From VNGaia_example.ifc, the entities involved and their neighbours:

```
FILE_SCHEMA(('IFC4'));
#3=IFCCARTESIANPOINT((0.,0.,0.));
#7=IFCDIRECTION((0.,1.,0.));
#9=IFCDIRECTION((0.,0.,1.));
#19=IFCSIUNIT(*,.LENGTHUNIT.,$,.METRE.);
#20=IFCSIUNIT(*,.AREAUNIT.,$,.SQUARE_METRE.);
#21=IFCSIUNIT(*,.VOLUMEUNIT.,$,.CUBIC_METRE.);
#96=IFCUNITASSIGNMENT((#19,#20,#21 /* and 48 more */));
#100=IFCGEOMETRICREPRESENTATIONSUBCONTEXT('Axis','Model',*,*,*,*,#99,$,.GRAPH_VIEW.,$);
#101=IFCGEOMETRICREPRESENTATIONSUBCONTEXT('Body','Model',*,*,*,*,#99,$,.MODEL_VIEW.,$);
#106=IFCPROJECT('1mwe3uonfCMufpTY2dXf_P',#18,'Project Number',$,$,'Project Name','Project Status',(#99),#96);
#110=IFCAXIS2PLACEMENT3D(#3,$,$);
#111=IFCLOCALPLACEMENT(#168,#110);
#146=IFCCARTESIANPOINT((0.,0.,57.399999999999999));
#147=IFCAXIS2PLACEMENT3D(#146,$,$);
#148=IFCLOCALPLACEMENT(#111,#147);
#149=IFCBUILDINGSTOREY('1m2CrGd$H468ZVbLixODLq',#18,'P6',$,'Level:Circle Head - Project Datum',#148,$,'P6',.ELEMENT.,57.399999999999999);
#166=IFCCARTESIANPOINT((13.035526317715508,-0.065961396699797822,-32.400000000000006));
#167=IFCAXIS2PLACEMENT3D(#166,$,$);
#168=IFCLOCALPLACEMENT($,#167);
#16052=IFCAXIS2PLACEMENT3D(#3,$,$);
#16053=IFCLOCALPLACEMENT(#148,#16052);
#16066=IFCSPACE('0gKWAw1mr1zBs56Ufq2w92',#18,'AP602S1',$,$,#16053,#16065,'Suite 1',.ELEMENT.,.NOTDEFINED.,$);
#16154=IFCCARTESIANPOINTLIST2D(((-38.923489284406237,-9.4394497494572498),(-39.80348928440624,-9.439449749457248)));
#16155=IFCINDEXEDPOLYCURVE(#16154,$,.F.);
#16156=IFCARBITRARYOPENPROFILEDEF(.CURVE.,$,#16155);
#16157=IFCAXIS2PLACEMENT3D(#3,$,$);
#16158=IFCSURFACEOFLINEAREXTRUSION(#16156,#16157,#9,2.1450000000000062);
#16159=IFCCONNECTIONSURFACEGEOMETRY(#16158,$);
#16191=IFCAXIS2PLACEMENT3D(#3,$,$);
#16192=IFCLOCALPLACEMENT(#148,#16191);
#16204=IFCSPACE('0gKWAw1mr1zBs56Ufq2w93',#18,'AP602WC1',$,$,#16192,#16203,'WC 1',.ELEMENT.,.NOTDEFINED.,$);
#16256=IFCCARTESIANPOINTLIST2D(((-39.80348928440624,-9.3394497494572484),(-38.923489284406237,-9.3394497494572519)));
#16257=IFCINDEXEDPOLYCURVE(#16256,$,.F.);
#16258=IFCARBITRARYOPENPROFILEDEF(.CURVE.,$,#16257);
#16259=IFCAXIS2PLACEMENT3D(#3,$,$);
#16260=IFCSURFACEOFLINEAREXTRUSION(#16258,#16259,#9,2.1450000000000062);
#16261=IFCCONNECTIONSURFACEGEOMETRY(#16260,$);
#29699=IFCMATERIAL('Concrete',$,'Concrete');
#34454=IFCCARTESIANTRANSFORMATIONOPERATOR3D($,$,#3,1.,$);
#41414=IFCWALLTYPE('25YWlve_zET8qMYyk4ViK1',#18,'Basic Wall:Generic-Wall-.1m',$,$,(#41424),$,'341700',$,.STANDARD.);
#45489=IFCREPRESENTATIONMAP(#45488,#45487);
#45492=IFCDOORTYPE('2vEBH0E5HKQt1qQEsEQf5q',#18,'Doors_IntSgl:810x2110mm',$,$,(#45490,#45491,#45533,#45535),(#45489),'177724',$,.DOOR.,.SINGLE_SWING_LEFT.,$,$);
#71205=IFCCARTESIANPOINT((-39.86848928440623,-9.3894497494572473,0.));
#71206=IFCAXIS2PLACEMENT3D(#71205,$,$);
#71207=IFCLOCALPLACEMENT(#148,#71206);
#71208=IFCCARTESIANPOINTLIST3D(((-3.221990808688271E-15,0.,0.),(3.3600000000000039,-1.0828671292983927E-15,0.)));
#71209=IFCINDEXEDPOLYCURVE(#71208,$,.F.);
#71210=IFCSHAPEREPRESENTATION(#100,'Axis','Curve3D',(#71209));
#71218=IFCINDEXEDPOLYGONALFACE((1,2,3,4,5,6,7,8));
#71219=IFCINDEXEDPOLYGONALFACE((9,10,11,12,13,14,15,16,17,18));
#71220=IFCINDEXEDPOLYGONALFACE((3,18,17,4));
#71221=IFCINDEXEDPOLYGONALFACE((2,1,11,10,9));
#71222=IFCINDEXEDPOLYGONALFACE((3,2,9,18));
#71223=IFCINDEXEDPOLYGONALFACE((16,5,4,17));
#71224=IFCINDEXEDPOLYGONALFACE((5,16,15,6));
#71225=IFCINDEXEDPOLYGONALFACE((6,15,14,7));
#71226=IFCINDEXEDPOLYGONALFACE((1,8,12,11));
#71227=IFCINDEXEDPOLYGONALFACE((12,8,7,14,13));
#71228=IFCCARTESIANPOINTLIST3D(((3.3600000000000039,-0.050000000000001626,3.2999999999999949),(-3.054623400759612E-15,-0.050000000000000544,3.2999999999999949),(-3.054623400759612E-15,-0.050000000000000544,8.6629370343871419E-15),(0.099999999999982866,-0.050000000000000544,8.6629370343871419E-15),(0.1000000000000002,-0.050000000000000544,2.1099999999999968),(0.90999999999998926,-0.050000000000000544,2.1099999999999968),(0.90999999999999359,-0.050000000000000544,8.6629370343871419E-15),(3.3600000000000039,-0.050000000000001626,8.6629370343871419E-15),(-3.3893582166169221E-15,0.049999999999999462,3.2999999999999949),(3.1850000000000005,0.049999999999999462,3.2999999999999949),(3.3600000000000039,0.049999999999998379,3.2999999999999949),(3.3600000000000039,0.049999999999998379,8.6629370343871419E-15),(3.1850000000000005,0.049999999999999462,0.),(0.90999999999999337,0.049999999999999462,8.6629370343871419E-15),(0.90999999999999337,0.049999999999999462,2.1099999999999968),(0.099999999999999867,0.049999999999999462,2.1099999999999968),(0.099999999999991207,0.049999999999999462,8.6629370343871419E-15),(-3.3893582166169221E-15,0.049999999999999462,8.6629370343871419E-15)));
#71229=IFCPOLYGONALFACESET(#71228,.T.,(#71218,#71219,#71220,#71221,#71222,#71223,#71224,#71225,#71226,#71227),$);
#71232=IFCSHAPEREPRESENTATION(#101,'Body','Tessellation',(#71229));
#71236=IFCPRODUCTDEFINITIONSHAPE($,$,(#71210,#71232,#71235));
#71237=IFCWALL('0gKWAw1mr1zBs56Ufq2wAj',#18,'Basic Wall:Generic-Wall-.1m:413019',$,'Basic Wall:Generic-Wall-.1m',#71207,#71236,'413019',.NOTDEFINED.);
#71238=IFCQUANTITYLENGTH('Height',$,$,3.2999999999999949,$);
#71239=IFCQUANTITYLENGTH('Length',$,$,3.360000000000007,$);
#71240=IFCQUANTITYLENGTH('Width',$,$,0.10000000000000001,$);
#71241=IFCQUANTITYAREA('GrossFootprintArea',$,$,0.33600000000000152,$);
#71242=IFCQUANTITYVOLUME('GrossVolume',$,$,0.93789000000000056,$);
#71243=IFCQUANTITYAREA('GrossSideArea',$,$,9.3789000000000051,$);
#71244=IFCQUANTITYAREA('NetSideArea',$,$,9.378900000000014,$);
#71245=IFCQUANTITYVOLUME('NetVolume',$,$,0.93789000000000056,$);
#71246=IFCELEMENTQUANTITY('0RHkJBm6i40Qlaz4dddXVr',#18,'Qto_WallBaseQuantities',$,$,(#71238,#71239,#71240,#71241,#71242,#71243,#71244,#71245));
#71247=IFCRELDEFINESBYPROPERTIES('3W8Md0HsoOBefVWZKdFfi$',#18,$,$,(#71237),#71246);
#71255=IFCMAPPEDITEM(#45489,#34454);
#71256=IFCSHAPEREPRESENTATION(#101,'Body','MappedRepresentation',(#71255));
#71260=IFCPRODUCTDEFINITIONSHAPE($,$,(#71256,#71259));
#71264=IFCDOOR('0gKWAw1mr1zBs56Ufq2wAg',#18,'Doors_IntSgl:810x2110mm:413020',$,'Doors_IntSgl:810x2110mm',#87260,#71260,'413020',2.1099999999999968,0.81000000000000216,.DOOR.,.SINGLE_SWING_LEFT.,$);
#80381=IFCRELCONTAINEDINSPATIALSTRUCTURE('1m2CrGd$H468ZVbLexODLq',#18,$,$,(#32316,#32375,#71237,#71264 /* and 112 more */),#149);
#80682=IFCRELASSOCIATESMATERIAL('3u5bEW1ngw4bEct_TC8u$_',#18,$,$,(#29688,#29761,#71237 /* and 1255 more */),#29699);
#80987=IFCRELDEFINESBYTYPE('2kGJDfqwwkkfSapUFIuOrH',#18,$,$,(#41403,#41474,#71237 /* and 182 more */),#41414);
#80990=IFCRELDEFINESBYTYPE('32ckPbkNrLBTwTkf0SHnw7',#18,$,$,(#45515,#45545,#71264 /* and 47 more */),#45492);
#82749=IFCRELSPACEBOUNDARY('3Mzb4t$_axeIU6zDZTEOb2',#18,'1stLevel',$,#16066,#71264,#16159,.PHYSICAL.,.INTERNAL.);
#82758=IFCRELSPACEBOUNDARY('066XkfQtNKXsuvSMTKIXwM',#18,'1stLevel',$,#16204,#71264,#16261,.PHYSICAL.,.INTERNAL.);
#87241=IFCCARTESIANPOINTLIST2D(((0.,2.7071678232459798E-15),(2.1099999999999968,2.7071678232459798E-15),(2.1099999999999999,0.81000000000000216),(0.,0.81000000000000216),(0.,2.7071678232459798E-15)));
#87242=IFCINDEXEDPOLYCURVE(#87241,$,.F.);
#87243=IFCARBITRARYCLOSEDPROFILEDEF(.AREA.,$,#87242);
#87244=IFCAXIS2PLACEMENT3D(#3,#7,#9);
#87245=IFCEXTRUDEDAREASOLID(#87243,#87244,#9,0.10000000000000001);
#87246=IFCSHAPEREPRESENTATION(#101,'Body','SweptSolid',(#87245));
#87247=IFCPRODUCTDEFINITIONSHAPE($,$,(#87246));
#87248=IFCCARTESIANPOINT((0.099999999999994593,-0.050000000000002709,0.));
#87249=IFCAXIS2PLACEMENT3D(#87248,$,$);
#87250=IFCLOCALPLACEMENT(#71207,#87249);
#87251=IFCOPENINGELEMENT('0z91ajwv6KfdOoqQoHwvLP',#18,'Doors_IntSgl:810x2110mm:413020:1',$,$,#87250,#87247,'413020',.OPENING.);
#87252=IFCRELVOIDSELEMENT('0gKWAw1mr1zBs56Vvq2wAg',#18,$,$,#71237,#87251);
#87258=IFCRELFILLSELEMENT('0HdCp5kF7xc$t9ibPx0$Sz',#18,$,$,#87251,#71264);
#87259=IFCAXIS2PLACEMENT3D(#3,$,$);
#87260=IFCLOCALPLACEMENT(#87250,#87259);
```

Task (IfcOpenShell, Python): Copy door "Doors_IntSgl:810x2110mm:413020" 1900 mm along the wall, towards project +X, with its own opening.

```python
import numpy as np
import ifcopenshell
import ifcopenshell.api.feature
import ifcopenshell.api.geometry
import ifcopenshell.api.pset
import ifcopenshell.api.root
import ifcopenshell.geom
import ifcopenshell.util.element
import ifcopenshell.util.placement
import ifcopenshell.util.shape
import ifcopenshell.util.unit

model = ifcopenshell.open("VNGaia_example.ifc")
area_scale = ifcopenshell.util.unit.calculate_unit_scale(model, "AREAUNIT")
volume_scale = ifcopenshell.util.unit.calculate_unit_scale(model, "VOLUMEUNIT")
settings = ifcopenshell.geom.settings()


def volume(element):
    """Net volume in cubic metres, openings subtracted."""
    shape = ifcopenshell.geom.create_shape(settings, element)
    return ifcopenshell.util.shape.get_volume(shape.geometry)


def reuse_history(source, copy):
    """copy_class also copies each property set's owner history, people and application; keep the originals."""
    for rel in copy.IsDefinedBy:
        if rel.is_a("IfcRelDefinesByProperties") and (history := rel.RelatingPropertyDefinition.OwnerHistory):
            rel.RelatingPropertyDefinition.OwnerHistory = source.OwnerHistory
            ifcopenshell.util.element.remove_deep2(model, history)


door = model.by_id(71264)
opening = door.FillsVoids[0].RelatingOpeningElement
wall = opening.VoidsElements[0].RelatingBuildingElement
before = volume(wall)
shift = ifcopenshell.util.placement.get_local_placement(wall.ObjectPlacement)[:3, 0] * 1.9

# copy_class copies the void relationship, type, container and properties, but no geometry.
new_opening = ifcopenshell.api.root.copy_class(model, product=opening)
new_opening.Representation = ifcopenshell.util.element.copy_deep(
    model, opening.Representation, exclude=["IfcGeometricRepresentationContext", "IfcRepresentationMap"]
)
new_opening.Name = "Doors_IntSgl:810x2110mm"
new_opening.Tag = None
reuse_history(opening, new_opening)
new_door = ifcopenshell.api.root.copy_class(model, product=door)
new_door.Representation = ifcopenshell.util.element.copy_deep(
    model, door.Representation, exclude=["IfcGeometricRepresentationContext", "IfcRepresentationMap"]
)
new_door.Name = "Doors_IntSgl:810x2110mm"
new_door.Tag = None
reuse_history(door, new_door)
ifcopenshell.api.feature.add_filling(model, opening=new_opening, element=new_door)

for old, new in ((opening, new_opening), (door, new_door)):
    matrix = ifcopenshell.util.placement.get_local_placement(old.ObjectPlacement)
    matrix[:3, 3] += shift
    ifcopenshell.api.geometry.edit_object_placement(model, product=new, matrix=matrix, is_si=False)

# The copied space boundaries still share their surfaces with the original.
for rel in new_door.ProvidesBoundaries:
    if rel.ConnectionGeometry:
        rel.ConnectionGeometry = ifcopenshell.util.element.copy_deep(model, rel.ConnectionGeometry)

# Space boundary surfaces are stored in each space's coordinates; move them too.
for rel in new_door.ProvidesBoundaries:
    if not rel.ConnectionGeometry:
        continue
    surface = rel.ConnectionGeometry.SurfaceOnRelatingElement
    space_matrix = ifcopenshell.util.placement.get_local_placement(rel.RelatingSpace.ObjectPlacement)
    point = np.array(surface.Position.Location.Coordinates) + space_matrix[:3, :3].T @ shift
    surface.Position = model.createIfcAxis2Placement3D(
        model.createIfcCartesianPoint(point.tolist()), surface.Position.Axis, surface.Position.RefDirection
    )

after = volume(wall)
thickness = 0.1  # wall thickness in metres

# Update the wall's stored quantities.
qto = model.by_id(ifcopenshell.util.element.get_pset(wall, "Qto_WallBaseQuantities", should_inherit=False)["id"])
ifcopenshell.api.pset.edit_qto(model, qto=qto, properties={
    "NetSideArea": after / thickness / area_scale,
    "NetVolume": after / volume_scale,
})

print(f"wall volume {before:.3f} -> {after:.3f} m3")

model.write("VNGaia_example_edited.ifc")
```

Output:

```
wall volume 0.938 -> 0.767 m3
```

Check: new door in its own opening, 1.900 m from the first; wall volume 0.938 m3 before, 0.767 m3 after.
